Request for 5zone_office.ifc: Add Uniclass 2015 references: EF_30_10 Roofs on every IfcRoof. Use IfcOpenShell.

First a look at what the model holds.

```python
import ifcopenshell

model = ifcopenshell.open("5zone_office.ifc")
print(model.schema)
print("classifications:", [c.Name for c in model.by_type("IfcClassification")])
for ifc_class in ("IfcDoor", "IfcRoof", "IfcStair", "IfcWall", "IfcWindow"):
    print(ifc_class, len(model.by_type(ifc_class)))
```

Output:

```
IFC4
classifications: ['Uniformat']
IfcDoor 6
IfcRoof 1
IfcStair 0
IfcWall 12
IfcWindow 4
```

```python
import ifcopenshell
import ifcopenshell.api.classification

model = ifcopenshell.open("5zone_office.ifc")

system = ifcopenshell.api.classification.add_classification(model, classification="Uniclass 2015")

codes = {
    "IfcRoof": ("EF_30_10", "Roofs"),
}
for ifc_class, (code, name) in codes.items():
    products = model.by_type(ifc_class)
    ifcopenshell.api.classification.add_reference(
        model, products=products, classification=system, identification=code, name=name
    )
    print(code, len(products))

model.write("5zone_office_rev.ifc")
```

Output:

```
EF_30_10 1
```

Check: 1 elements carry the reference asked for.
